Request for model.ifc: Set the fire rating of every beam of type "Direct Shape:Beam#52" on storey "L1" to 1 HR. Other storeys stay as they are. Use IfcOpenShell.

First a look at what the model holds.

```python
import ifcopenshell
import ifcopenshell.util.element

model = ifcopenshell.open("model.ifc")
print(model.schema)
storey = next(s for s in model.by_type("IfcBuildingStorey") if s.Name == "L1")
beams = [e for e in ifcopenshell.util.element.get_decomposition(storey) if e.is_a("IfcBeam")]
seen = {}
for e in beams:
    element_type = ifcopenshell.util.element.get_type(e)
    key = (element_type.Name if element_type != e and element_type else None, ifcopenshell.util.element.get_pset(e, "Pset_BeamCommon", "FireRating"))
    seen[key] = seen.get(key, 0) + 1
for (name, value), count in sorted(seen.items(), key=str):
    print(count, "x", name, "|", value)
```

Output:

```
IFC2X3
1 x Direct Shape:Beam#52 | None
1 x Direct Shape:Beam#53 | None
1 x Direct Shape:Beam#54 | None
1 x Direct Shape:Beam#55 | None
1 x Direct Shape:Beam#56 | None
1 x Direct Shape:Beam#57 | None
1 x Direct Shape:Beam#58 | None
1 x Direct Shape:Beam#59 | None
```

```python
import ifcopenshell
import ifcopenshell.api.pset
import ifcopenshell.util.element

model = ifcopenshell.open("model.ifc")

storey = next(s for s in model.by_type("IfcBuildingStorey") if s.Name == "L1")
beams = [e for e in ifcopenshell.util.element.get_decomposition(storey) if e.is_a("IfcBeam")]

count = 0
for e in beams:
    element_type = ifcopenshell.util.element.get_type(e)
    if element_type in (None, e) or element_type.Name != "Direct Shape:Beam#52":
        continue
    # add_pset returns the element's existing set when there is one.
    pset = ifcopenshell.api.pset.add_pset(model, product=e, name="Pset_BeamCommon")
    ifcopenshell.api.pset.edit_pset(model, pset=pset, properties={"FireRating": "1 HR"})
    count += 1

print(count, "beams updated")

model.write("model_edited.ifc")
```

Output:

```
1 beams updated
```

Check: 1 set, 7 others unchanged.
